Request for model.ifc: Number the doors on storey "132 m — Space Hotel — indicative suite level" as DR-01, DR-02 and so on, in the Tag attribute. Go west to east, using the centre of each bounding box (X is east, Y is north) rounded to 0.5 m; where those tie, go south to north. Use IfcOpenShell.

First a look at what the model holds.

```python
import ifcopenshell
import ifcopenshell.util.element
import ifcopenshell.util.placement

model = ifcopenshell.open("model.ifc")
print(model.schema)
storey = next(s for s in model.by_type("IfcBuildingStorey") if s.Name == "132 m — Space Hotel — indicative suite level")
doors = [e for e in ifcopenshell.util.element.get_decomposition(storey) if e.is_a("IfcDoor")]
for e in sorted(doors, key=lambda e: e.id()):
    origin = ifcopenshell.util.placement.get_local_placement(e.ObjectPlacement)[:3, 3]
    print(e.id(), e.Tag, e.Name, origin.round(2) + 0.0, sep=" | ")
```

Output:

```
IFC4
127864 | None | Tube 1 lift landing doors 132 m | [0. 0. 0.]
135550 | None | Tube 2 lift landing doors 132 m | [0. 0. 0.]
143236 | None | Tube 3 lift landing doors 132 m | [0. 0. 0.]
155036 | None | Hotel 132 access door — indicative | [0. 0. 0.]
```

```python
import ifcopenshell
import ifcopenshell.geom
import ifcopenshell.util.element
import ifcopenshell.util.shape

model = ifcopenshell.open("model.ifc")
settings = ifcopenshell.geom.settings()
settings.set("use-world-coords", True)


def centre(element):
    shape = ifcopenshell.geom.create_shape(settings, element)
    return ifcopenshell.util.shape.get_bbox_centroid(shape.geometry)


storey = next(s for s in model.by_type("IfcBuildingStorey") if s.Name == "132 m — Space Hotel — indicative suite level")
doors = [e for e in ifcopenshell.util.element.get_decomposition(storey) if e.is_a("IfcDoor")]

# Insertion points can sit at a corner or the storey origin, so sort by the geometry (in metres).
centres = {e: centre(e) for e in doors}
doors.sort(key=lambda e: (round(centres[e][0] / 0.5), centres[e][1]))

for i, e in enumerate(doors, start=1):
    number = f"DR-{i:02d}"
    e.Tag = number
    print(e.id(), number)

model.write("model_v2.ifc")
```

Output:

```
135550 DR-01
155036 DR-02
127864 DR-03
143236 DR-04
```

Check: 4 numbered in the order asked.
